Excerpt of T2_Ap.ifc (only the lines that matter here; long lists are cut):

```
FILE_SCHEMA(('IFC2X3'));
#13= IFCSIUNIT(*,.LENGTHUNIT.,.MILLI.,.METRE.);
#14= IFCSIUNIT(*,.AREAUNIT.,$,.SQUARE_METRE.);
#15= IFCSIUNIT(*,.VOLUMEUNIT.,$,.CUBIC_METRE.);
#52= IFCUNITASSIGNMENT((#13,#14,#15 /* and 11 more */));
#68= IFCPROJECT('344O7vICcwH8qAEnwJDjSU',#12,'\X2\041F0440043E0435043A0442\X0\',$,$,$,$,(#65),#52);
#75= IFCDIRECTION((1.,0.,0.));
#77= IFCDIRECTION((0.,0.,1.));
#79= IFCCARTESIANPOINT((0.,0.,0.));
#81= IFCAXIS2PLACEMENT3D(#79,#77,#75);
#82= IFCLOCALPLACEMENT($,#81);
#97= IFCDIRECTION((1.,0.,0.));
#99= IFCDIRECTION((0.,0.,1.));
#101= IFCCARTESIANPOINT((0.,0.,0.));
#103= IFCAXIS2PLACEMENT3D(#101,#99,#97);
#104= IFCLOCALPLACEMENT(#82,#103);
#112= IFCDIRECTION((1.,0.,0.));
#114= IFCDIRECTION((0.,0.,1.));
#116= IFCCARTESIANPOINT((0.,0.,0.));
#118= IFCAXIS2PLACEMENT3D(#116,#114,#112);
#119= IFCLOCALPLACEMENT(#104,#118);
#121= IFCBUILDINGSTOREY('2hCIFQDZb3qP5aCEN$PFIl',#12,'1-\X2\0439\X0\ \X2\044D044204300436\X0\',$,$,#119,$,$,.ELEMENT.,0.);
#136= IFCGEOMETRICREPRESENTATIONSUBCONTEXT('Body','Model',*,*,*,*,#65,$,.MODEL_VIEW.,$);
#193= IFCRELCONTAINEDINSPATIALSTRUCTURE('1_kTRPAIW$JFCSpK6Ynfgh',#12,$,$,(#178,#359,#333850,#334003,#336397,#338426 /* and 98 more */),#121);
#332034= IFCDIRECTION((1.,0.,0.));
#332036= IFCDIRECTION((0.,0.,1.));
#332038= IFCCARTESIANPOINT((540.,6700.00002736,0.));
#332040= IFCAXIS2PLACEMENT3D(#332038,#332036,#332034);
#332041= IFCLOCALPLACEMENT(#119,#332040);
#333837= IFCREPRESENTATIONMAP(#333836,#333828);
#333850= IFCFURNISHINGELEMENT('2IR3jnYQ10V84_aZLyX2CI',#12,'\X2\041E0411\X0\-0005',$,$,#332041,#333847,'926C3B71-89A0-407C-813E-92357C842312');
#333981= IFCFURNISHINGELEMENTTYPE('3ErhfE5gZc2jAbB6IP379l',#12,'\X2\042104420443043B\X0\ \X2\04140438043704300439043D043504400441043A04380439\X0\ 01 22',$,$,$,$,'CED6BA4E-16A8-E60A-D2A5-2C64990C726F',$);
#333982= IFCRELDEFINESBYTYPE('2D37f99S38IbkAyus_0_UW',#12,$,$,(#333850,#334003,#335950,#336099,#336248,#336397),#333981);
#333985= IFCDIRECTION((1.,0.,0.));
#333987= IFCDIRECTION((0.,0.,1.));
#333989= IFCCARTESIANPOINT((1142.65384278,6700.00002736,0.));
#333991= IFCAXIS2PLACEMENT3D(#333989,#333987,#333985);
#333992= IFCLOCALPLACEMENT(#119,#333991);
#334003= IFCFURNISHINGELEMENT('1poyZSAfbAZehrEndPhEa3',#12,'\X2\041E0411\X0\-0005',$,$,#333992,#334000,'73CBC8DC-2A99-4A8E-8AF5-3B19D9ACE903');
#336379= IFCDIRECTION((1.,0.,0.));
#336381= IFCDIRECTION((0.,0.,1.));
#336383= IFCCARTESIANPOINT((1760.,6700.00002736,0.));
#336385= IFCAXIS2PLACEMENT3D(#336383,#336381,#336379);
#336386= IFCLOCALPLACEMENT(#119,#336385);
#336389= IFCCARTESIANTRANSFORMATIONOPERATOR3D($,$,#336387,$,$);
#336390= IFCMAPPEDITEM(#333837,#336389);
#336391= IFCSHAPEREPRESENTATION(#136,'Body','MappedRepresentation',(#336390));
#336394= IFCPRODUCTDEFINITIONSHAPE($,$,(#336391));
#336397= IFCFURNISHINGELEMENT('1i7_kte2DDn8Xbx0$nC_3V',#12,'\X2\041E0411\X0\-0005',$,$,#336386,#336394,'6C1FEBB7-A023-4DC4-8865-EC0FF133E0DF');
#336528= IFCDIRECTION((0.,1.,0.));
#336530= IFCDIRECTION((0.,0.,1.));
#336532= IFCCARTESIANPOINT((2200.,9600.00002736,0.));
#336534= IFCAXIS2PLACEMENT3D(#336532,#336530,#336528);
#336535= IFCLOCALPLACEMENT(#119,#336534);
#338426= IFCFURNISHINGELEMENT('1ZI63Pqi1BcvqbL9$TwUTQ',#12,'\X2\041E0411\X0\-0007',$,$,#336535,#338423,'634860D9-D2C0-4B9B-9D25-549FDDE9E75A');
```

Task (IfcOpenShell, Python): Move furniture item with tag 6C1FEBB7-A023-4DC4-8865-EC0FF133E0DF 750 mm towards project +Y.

```python
import ifcopenshell
import ifcopenshell.api.geometry
import ifcopenshell.util.placement

model = ifcopenshell.open("T2_Ap.ifc")

item = model.by_guid("1i7_kte2DDn8Xbx0$nC_3V")
matrix = ifcopenshell.util.placement.get_local_placement(item.ObjectPlacement)
matrix[1, 3] += 750.0
ifcopenshell.api.geometry.edit_object_placement(model, product=item, matrix=matrix, is_si=False)

print(ifcopenshell.util.placement.get_local_placement(item.ObjectPlacement).round(3) + 0.0)

model.write("T2_Ap-out.ifc")
```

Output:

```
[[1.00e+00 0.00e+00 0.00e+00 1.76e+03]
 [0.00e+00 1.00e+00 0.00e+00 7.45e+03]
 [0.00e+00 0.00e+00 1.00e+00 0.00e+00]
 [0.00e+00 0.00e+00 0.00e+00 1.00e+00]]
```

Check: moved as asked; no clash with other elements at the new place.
